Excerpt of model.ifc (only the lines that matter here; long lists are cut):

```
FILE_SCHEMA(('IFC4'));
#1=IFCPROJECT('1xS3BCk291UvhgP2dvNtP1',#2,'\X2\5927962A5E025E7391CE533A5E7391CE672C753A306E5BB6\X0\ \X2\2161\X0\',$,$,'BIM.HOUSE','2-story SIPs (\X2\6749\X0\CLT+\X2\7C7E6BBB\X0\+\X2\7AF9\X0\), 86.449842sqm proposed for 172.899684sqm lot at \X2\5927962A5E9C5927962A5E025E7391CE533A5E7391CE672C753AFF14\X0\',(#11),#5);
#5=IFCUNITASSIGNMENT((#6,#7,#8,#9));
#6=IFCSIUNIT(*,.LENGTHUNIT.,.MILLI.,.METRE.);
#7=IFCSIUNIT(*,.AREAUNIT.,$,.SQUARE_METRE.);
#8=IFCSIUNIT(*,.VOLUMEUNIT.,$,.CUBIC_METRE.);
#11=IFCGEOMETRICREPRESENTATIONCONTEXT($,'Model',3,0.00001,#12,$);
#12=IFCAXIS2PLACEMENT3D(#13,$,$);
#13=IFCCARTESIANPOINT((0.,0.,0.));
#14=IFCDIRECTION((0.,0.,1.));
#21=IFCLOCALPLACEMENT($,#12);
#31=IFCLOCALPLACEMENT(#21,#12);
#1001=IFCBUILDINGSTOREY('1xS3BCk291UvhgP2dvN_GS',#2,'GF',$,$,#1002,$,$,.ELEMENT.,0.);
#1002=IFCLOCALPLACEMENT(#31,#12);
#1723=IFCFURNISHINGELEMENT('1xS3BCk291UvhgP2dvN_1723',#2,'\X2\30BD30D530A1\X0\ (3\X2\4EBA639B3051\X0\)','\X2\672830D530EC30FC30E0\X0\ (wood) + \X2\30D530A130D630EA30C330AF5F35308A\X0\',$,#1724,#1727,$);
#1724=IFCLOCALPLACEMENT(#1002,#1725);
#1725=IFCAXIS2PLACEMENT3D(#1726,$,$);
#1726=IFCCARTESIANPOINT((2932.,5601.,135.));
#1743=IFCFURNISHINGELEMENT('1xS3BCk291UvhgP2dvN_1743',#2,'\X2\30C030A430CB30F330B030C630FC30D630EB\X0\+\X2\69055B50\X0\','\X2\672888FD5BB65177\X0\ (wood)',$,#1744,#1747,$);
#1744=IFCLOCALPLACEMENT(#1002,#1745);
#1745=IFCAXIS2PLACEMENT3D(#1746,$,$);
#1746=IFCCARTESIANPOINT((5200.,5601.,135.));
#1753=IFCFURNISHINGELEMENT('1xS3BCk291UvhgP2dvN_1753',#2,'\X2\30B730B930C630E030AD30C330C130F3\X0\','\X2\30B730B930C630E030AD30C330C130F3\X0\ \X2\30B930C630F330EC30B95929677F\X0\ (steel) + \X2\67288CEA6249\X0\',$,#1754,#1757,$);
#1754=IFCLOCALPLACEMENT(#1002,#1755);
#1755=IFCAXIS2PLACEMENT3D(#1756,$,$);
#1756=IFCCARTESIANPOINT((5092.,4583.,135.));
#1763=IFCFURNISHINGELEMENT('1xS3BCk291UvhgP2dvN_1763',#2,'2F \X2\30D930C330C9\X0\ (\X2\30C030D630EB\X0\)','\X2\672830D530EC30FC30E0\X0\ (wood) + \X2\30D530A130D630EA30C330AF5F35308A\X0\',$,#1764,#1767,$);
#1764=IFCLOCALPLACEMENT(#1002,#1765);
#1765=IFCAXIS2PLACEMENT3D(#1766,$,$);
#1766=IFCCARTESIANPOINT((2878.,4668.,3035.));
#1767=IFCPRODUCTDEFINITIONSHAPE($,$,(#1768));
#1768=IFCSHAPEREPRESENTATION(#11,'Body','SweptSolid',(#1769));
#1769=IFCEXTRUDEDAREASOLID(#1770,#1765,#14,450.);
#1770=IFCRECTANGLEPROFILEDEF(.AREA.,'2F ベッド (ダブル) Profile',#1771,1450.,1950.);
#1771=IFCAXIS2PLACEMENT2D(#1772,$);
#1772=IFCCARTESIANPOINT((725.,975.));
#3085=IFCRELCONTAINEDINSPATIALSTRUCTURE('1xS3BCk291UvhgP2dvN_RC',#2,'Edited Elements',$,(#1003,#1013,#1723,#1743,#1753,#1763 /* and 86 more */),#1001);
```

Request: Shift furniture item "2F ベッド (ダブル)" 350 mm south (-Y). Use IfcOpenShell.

```python
import ifcopenshell
import ifcopenshell.api.geometry
import ifcopenshell.util.placement

model = ifcopenshell.open("model.ifc")

item = model.by_guid("1xS3BCk291UvhgP2dvN_1763")
matrix = ifcopenshell.util.placement.get_local_placement(item.ObjectPlacement)
matrix[1, 3] -= 350.0
ifcopenshell.api.geometry.edit_object_placement(model, product=item, matrix=matrix, is_si=False)

print(ifcopenshell.util.placement.get_local_placement(item.ObjectPlacement).round(3) + 0.0)

model.write("model_edited.ifc")
```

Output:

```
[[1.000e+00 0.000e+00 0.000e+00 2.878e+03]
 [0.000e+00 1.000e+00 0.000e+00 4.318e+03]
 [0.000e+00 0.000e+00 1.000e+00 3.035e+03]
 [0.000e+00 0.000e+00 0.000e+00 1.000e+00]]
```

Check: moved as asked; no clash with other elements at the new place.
